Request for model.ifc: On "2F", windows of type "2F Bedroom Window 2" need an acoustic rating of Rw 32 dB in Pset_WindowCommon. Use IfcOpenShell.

First a look at what the model holds.

```python
import ifcopenshell
import ifcopenshell.util.element

model = ifcopenshell.open("model.ifc")
print(model.schema)
storey = next(s for s in model.by_type("IfcBuildingStorey") if s.Name == "2F")
windows = [e for e in ifcopenshell.util.element.get_decomposition(storey) if e.is_a("IfcWindow")]
seen = {}
for e in windows:
    element_type = ifcopenshell.util.element.get_type(e)
    key = (element_type.Name if element_type != e and element_type else None, ifcopenshell.util.element.get_pset(e, "Pset_WindowCommon", "AcousticRating"))
    seen[key] = seen.get(key, 0) + 1
for (name, value), count in sorted(seen.items(), key=str):
    print(count, "x", name, "|", value)
```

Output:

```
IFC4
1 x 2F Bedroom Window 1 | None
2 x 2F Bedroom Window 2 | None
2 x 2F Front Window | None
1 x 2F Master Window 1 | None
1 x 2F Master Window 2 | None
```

```python
import ifcopenshell
import ifcopenshell.api.pset
import ifcopenshell.util.element

model = ifcopenshell.open("model.ifc")

storey = next(s for s in model.by_type("IfcBuildingStorey") if s.Name == "2F")
windows = [e for e in ifcopenshell.util.element.get_decomposition(storey) if e.is_a("IfcWindow")]

count = 0
for e in windows:
    element_type = ifcopenshell.util.element.get_type(e)
    if element_type in (None, e) or element_type.Name != "2F Bedroom Window 2":
        continue
    # add_pset returns the element's existing set when there is one.
    pset = ifcopenshell.api.pset.add_pset(model, product=e, name="Pset_WindowCommon")
    ifcopenshell.api.pset.edit_pset(model, pset=pset, properties={"AcousticRating": "Rw 32 dB"})
    count += 1

print(count, "windows updated")

model.write("model_rev.ifc")
```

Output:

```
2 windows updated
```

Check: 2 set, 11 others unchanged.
